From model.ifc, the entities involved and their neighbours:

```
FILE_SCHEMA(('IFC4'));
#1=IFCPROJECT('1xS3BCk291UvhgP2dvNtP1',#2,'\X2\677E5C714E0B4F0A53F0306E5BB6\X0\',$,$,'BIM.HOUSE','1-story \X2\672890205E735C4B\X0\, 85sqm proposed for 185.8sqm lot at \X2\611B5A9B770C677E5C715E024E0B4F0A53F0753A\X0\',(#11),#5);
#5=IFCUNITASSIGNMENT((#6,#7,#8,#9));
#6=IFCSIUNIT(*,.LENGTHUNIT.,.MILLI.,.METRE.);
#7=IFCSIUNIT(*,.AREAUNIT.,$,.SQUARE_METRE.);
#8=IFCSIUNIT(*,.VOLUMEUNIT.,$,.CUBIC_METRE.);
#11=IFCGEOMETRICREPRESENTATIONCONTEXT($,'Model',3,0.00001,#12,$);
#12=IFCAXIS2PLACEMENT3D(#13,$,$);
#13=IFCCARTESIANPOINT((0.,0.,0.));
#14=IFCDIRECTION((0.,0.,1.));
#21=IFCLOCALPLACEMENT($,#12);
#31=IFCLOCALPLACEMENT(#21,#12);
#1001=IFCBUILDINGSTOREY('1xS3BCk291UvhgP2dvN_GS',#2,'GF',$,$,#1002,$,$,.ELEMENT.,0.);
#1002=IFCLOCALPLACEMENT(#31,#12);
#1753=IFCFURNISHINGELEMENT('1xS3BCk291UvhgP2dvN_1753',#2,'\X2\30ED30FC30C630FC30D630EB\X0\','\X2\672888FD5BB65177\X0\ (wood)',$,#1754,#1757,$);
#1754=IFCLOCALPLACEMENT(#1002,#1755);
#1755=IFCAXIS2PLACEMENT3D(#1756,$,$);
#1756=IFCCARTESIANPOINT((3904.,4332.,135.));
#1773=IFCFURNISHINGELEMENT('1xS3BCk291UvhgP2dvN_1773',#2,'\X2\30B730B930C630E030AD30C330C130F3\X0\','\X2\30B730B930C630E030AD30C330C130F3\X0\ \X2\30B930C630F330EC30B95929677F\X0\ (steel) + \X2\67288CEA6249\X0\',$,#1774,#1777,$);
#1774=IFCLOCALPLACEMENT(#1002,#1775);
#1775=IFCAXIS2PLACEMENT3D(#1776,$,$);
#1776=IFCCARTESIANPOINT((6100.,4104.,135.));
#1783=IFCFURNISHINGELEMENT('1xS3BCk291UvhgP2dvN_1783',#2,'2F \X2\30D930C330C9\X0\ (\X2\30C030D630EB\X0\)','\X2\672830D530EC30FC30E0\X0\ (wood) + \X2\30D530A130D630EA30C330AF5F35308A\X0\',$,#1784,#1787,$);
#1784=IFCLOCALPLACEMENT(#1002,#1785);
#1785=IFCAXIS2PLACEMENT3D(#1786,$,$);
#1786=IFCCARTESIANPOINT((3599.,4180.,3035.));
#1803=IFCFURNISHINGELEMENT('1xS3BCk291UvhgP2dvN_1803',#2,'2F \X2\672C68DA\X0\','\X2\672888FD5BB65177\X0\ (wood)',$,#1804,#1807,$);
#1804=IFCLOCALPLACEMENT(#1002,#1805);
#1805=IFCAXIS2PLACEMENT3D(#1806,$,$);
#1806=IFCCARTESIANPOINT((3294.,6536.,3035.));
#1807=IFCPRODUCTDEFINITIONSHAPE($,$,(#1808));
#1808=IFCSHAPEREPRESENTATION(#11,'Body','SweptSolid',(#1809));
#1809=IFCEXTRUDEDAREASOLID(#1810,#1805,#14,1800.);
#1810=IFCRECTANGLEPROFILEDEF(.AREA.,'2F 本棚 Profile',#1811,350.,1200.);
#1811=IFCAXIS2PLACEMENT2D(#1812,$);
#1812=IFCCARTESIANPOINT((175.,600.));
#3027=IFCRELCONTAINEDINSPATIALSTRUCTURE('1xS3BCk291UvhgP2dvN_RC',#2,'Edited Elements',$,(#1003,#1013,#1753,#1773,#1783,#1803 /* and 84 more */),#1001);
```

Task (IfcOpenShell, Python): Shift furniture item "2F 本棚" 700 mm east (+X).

```python
import ifcopenshell
import ifcopenshell.api.geometry
import ifcopenshell.util.placement

model = ifcopenshell.open("model.ifc")

item = model.by_guid("1xS3BCk291UvhgP2dvN_1803")
matrix = ifcopenshell.util.placement.get_local_placement(item.ObjectPlacement)
matrix[0, 3] += 700.0
ifcopenshell.api.geometry.edit_object_placement(model, product=item, matrix=matrix, is_si=False)

print(ifcopenshell.util.placement.get_local_placement(item.ObjectPlacement).round(3) + 0.0)

model.write("model_rev.ifc")
```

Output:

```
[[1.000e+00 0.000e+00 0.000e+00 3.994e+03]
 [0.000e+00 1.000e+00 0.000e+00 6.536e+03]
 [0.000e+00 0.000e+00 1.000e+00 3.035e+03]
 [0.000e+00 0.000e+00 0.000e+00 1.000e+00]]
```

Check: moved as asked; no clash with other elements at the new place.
